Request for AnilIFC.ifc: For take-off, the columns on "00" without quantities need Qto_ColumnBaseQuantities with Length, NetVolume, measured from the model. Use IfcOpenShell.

First a look at what the model holds.

```python
import ifcopenshell
import ifcopenshell.util.element
import ifcopenshell.util.unit

model = ifcopenshell.open("AnilIFC.ifc")
print(model.schema)
for unit_type in ("LENGTHUNIT", "AREAUNIT", "VOLUMEUNIT"):
    print(unit_type, ifcopenshell.util.unit.calculate_unit_scale(model, unit_type))
storey = next(s for s in model.by_type("IfcBuildingStorey") if s.Name == "00")
columns = [e for e in ifcopenshell.util.element.get_decomposition(storey) if e.is_a("IfcColumn")]
for e in sorted(columns, key=lambda e: e.id()):
    print(e.id(), e.is_a(), e.Name, list(ifcopenshell.util.element.get_psets(e, qtos_only=True)), sep=" | ")
```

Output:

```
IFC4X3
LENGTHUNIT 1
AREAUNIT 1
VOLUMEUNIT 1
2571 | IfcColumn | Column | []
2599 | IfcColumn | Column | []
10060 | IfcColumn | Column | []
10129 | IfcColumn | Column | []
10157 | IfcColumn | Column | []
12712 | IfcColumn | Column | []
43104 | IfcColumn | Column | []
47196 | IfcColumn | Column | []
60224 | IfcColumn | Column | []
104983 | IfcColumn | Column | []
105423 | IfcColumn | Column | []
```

```python
import ifcopenshell
import ifcopenshell.api.pset
import ifcopenshell.geom
import ifcopenshell.util.element
import ifcopenshell.util.shape
import ifcopenshell.util.unit

model = ifcopenshell.open("AnilIFC.ifc")
unit_scale = ifcopenshell.util.unit.calculate_unit_scale(model)
volume_scale = ifcopenshell.util.unit.calculate_unit_scale(model, "VOLUMEUNIT")
settings = ifcopenshell.geom.settings()

storey = next(s for s in model.by_type("IfcBuildingStorey") if s.Name == "00")
columns = [e for e in ifcopenshell.util.element.get_decomposition(storey) if e.is_a("IfcColumn")]

for e in sorted(columns, key=lambda e: e.id()):
    if ifcopenshell.util.element.get_psets(e, qtos_only=True, should_inherit=False):
        continue
    # Geometry comes back in metres, in the element's own axes.
    shape = ifcopenshell.geom.create_shape(settings, e)
    values = {
        "Length": ifcopenshell.util.shape.get_z(shape.geometry) / unit_scale,
        "NetVolume": ifcopenshell.util.shape.get_volume(shape.geometry) / volume_scale,
    }
    qto = ifcopenshell.api.pset.add_qto(model, product=e, name="Qto_ColumnBaseQuantities")
    ifcopenshell.api.pset.edit_qto(model, qto=qto, properties=values)
    print(e.id(), {k: round(v, 3) for k, v in values.items()})

model.write("AnilIFC_updated.ifc")
```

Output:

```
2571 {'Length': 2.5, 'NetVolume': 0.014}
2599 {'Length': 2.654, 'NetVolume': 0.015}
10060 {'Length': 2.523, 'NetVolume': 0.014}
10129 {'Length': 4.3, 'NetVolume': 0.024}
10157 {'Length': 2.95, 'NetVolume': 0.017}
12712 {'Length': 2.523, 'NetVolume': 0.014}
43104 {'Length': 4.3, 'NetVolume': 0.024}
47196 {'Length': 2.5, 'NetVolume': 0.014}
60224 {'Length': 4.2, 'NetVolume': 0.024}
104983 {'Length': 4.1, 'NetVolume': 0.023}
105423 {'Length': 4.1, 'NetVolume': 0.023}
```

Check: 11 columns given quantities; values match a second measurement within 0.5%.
